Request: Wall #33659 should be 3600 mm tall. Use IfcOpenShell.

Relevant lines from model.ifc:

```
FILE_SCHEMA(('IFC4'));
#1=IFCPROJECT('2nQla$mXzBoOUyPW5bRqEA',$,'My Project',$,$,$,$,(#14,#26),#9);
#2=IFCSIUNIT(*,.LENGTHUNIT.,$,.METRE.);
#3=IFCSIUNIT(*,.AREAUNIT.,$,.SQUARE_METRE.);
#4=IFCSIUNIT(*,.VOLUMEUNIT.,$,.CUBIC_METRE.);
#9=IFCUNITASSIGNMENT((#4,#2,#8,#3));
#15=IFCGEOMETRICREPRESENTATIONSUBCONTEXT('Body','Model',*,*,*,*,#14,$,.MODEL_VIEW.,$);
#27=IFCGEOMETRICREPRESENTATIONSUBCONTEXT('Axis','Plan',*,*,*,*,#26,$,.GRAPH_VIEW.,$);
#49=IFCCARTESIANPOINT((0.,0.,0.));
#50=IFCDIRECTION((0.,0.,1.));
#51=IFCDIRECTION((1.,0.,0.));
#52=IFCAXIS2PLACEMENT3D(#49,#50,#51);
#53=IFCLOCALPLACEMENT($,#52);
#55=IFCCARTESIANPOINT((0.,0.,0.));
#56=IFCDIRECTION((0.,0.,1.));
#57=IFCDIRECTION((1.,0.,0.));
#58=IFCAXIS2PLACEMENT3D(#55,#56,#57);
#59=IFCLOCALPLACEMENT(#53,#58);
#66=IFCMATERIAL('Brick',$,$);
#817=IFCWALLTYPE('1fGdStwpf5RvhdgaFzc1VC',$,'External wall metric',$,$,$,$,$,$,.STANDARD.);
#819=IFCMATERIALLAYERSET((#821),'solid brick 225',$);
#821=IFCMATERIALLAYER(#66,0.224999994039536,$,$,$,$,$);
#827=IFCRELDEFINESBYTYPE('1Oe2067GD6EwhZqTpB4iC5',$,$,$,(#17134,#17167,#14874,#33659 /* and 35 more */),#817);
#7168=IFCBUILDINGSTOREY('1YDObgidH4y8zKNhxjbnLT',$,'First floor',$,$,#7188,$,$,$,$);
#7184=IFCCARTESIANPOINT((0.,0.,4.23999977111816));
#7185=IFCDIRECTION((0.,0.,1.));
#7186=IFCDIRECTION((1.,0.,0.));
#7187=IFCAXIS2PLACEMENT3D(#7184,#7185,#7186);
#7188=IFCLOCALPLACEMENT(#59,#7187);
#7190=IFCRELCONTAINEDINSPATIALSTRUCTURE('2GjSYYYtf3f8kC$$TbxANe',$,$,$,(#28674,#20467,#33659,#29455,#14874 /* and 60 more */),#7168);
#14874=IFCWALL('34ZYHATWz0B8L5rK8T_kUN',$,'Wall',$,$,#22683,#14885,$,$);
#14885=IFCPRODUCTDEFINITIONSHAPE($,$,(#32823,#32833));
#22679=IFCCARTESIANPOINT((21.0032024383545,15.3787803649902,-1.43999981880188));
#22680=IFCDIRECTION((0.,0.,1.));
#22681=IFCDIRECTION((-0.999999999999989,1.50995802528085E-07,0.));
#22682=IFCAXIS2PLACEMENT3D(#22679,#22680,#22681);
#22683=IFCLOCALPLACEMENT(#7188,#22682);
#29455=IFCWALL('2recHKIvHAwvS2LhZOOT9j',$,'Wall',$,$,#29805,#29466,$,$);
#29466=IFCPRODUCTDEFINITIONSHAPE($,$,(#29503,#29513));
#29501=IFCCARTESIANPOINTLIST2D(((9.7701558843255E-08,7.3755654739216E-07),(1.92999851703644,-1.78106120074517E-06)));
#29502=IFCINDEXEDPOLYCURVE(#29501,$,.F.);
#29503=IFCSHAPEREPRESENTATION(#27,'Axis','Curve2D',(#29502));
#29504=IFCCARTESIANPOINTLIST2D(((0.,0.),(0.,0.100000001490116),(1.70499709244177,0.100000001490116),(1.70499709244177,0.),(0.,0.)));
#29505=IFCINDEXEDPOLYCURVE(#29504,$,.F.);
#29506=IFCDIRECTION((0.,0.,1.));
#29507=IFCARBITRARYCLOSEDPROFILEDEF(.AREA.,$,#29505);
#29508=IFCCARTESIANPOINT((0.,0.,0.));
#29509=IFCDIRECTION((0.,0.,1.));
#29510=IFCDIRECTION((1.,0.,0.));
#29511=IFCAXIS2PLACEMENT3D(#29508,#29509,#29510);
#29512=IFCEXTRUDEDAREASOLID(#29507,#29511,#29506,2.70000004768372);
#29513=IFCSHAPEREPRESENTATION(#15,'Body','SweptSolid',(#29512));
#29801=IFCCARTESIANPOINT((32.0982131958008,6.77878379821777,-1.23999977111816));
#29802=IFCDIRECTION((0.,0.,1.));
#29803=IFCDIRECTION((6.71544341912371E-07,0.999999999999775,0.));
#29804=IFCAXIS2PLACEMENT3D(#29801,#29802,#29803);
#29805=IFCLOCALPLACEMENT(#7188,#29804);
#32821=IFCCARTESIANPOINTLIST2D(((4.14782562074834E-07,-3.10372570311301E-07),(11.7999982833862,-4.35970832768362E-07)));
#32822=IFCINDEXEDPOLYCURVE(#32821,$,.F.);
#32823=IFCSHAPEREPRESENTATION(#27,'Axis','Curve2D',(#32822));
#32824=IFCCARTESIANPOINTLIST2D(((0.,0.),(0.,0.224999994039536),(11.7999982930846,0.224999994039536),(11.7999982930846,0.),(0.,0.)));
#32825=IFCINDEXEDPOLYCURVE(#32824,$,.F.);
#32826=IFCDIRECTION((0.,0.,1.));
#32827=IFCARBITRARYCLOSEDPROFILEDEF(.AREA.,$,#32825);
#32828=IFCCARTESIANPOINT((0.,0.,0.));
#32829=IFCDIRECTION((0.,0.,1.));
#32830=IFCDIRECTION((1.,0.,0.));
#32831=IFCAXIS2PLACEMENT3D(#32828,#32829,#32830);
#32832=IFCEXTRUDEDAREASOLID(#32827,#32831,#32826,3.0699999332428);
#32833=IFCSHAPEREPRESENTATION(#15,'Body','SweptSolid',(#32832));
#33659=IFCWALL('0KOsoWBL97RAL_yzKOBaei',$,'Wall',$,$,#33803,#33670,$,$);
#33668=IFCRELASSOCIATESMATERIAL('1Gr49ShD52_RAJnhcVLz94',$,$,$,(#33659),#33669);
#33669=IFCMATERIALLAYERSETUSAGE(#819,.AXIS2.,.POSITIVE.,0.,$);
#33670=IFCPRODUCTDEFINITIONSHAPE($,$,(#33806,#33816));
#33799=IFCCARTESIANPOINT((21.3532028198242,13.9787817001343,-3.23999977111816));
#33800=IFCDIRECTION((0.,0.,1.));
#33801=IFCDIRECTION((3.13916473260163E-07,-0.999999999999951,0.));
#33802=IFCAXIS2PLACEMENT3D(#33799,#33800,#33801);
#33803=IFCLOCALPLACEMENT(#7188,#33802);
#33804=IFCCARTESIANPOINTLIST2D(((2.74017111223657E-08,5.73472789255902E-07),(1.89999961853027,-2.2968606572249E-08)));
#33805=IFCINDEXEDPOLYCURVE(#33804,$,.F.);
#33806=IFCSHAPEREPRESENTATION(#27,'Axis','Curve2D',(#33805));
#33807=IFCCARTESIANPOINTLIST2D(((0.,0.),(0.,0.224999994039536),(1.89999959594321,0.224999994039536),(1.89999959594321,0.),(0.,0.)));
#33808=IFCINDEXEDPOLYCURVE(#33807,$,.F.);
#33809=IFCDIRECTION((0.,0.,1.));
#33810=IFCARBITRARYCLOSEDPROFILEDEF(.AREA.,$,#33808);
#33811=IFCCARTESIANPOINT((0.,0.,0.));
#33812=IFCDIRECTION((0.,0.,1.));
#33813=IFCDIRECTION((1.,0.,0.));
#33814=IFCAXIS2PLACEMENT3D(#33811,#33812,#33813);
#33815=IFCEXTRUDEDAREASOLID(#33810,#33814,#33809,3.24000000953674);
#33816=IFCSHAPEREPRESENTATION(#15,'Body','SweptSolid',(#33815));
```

```python
import ifcopenshell
import ifcopenshell.geom
import ifcopenshell.util.representation
import ifcopenshell.util.shape
import ifcopenshell.util.unit

model = ifcopenshell.open("model.ifc")
unit_scale = ifcopenshell.util.unit.calculate_unit_scale(model)
settings = ifcopenshell.geom.settings()


def volume(element):
    """Net volume in cubic metres, openings subtracted."""
    shape = ifcopenshell.geom.create_shape(settings, element)
    return ifcopenshell.util.shape.get_volume(shape.geometry)


wall = model.by_id(33659)
before = volume(wall)

body = ifcopenshell.util.representation.get_representation(wall, "Model", "Body")
solid = body.Items[0]
old_height = solid.Depth
solid.Depth = 3.6 / unit_scale
after = volume(wall)

print(f"height {old_height:g} -> {solid.Depth:g}, volume {before:.3f} -> {after:.3f} m3")

model.write("model_edited.ifc")
```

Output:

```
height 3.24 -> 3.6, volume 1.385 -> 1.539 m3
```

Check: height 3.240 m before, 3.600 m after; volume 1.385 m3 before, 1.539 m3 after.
